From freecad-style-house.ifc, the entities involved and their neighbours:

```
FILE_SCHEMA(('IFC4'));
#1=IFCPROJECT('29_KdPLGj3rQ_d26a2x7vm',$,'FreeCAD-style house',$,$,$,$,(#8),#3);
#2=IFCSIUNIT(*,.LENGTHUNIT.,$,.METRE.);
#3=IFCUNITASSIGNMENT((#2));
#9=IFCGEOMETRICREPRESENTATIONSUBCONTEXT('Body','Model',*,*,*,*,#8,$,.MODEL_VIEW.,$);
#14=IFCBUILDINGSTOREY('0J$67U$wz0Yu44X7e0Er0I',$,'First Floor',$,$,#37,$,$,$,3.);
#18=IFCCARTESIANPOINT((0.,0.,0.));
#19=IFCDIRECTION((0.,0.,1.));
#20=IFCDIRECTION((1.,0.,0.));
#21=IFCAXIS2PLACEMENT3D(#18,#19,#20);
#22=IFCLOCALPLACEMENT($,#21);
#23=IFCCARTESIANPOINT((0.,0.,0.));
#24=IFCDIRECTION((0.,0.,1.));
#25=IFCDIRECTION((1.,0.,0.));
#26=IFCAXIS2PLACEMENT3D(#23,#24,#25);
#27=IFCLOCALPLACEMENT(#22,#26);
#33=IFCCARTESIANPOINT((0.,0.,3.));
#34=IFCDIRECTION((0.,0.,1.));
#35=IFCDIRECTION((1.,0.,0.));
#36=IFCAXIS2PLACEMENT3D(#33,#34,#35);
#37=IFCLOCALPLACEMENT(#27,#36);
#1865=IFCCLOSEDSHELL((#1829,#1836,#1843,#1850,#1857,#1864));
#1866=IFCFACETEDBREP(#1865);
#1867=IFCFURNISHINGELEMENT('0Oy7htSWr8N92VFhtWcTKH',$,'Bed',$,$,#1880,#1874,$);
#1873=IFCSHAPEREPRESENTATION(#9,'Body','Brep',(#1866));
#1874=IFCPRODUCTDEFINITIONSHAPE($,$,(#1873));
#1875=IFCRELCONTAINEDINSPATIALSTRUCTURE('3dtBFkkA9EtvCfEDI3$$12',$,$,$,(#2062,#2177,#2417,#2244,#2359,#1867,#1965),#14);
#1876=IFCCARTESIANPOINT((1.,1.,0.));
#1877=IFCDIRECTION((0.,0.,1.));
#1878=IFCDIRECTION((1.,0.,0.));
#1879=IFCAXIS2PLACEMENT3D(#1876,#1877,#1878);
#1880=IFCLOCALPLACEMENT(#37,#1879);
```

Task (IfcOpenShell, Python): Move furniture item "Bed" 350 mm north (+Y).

```python
import ifcopenshell
import ifcopenshell.api.geometry
import ifcopenshell.util.placement

model = ifcopenshell.open("freecad-style-house.ifc")

item = model.by_id(1867)
matrix = ifcopenshell.util.placement.get_local_placement(item.ObjectPlacement)
matrix[1, 3] += 0.35
ifcopenshell.api.geometry.edit_object_placement(model, product=item, matrix=matrix, is_si=False)

print(ifcopenshell.util.placement.get_local_placement(item.ObjectPlacement).round(3) + 0.0)

model.write("freecad-style-house_updated.ifc")
```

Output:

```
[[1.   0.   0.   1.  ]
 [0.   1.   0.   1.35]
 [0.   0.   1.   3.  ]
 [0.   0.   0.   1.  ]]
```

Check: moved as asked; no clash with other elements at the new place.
